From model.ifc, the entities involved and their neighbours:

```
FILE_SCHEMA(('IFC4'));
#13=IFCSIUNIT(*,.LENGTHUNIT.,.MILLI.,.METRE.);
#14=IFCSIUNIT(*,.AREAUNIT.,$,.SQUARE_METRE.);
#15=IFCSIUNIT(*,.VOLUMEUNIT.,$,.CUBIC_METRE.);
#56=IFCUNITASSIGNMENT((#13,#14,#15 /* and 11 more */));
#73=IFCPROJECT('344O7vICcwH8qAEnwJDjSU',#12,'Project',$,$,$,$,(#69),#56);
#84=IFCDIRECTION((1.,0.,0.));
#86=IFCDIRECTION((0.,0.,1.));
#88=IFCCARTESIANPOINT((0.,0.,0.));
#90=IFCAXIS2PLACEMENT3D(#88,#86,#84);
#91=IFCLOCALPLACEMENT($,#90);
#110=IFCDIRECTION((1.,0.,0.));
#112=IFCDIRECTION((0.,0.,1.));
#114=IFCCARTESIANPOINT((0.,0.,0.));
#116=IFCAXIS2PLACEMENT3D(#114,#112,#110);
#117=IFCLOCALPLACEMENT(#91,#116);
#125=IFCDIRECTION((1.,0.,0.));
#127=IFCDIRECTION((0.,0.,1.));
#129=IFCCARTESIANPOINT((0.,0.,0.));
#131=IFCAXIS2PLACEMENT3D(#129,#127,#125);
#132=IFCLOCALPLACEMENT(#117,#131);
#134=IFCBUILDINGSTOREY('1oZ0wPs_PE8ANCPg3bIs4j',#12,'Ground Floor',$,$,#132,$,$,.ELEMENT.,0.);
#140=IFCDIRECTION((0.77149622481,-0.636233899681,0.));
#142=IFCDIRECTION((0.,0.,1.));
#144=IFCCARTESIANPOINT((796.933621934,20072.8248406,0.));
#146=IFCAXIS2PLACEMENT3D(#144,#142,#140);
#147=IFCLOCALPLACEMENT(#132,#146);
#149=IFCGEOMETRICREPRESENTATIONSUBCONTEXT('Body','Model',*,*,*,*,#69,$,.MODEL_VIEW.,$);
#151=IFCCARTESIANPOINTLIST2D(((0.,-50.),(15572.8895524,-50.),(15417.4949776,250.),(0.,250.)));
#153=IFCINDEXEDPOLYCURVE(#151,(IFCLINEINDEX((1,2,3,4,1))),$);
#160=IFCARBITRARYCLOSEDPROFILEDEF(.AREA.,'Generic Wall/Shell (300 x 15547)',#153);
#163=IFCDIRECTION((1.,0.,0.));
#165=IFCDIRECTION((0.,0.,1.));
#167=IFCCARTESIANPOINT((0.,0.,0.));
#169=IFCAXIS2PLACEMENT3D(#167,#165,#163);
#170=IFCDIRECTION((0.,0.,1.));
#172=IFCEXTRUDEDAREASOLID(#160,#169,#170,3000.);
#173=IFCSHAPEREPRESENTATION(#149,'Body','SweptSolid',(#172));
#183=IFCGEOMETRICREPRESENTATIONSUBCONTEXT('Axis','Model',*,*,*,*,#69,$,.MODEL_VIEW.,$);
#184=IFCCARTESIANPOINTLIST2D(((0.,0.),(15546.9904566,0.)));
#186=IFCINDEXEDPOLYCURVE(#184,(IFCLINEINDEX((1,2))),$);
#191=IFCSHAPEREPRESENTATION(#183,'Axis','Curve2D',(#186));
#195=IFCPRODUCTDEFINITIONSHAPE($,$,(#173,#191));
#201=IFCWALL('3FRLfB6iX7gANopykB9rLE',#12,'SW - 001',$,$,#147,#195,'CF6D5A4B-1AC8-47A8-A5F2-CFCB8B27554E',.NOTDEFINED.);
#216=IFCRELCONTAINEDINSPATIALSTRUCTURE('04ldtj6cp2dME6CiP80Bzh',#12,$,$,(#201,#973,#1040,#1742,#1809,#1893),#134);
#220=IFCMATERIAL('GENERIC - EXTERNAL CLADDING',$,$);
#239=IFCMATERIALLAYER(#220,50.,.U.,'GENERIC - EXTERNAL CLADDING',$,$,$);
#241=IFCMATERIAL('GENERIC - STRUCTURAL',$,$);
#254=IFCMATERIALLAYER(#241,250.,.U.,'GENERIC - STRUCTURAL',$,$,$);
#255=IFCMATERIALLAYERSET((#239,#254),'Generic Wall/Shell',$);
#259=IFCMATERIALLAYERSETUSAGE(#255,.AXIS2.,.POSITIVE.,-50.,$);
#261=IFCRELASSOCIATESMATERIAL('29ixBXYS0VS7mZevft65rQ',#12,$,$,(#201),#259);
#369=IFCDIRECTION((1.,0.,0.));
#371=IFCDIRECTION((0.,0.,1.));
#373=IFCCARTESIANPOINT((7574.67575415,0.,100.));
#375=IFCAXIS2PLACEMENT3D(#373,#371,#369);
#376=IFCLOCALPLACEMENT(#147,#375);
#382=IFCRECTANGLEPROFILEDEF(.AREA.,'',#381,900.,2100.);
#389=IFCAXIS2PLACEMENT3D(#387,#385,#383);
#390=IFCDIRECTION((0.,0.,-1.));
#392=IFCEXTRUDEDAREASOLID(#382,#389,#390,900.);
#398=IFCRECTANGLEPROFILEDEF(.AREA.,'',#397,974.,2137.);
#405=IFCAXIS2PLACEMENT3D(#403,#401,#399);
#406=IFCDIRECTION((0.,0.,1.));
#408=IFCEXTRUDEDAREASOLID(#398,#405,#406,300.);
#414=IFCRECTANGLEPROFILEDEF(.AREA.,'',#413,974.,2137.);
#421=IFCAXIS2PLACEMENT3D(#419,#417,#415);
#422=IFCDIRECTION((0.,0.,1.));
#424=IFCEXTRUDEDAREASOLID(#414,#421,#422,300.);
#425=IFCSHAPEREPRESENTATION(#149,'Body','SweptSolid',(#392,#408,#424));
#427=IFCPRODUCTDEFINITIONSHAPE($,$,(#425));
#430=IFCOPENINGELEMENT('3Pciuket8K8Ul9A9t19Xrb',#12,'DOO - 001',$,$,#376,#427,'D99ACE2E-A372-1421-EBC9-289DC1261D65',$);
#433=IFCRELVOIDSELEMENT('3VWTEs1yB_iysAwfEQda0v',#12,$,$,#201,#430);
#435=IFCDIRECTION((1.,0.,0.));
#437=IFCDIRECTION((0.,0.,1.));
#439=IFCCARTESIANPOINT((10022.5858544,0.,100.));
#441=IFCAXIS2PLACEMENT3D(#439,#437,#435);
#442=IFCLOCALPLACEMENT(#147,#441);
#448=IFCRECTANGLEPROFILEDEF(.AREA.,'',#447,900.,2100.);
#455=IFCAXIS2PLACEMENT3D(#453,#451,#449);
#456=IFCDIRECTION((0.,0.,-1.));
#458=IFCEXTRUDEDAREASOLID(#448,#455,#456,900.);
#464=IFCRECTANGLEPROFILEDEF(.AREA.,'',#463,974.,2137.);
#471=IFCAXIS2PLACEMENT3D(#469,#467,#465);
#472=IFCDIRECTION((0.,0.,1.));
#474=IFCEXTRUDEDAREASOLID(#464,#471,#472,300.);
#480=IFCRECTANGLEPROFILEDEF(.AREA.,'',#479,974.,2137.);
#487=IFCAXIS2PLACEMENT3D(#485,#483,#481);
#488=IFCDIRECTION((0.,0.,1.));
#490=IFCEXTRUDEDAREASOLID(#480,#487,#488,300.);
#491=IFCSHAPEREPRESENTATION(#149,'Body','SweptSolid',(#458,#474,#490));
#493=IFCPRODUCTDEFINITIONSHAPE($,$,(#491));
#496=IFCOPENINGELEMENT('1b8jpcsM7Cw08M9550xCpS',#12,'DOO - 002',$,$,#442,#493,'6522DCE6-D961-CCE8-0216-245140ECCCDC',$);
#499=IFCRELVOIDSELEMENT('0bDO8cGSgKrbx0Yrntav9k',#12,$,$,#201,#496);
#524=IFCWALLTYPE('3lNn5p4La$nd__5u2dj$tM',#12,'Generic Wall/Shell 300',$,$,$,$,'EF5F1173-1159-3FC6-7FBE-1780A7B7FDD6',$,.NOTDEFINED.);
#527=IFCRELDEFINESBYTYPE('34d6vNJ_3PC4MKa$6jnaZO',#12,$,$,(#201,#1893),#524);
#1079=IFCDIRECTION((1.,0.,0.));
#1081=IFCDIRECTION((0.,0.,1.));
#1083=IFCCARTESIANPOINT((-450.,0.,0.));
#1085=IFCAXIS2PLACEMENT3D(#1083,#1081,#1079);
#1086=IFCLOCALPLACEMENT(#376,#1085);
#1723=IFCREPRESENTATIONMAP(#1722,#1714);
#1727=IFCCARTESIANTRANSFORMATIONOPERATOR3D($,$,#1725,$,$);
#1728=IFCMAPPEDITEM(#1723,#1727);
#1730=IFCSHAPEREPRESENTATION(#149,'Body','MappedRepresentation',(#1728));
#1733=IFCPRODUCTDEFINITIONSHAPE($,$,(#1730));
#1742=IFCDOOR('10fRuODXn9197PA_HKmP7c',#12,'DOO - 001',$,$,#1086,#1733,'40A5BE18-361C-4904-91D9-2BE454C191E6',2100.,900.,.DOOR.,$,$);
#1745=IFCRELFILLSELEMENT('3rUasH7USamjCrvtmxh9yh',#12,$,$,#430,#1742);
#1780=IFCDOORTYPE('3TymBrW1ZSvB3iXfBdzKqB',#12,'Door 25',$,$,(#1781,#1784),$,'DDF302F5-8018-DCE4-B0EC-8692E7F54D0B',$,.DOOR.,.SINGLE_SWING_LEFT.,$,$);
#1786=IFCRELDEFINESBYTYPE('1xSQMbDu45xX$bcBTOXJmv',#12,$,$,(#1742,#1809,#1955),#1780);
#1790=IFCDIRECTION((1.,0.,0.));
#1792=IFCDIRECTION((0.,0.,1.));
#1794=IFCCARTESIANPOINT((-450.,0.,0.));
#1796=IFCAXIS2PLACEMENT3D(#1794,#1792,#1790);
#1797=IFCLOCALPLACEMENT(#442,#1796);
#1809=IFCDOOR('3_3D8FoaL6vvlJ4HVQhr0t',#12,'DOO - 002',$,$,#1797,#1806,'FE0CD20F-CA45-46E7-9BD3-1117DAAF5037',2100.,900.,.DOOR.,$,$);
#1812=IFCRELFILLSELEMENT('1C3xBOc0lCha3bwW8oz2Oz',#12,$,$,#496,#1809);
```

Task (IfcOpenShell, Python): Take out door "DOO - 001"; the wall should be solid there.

```python
import ifcopenshell
import ifcopenshell.api.feature
import ifcopenshell.api.root
import ifcopenshell.geom
import ifcopenshell.util.shape

model = ifcopenshell.open("model.ifc")
settings = ifcopenshell.geom.settings()


def volume(element):
    """Net volume in cubic metres, openings subtracted."""
    shape = ifcopenshell.geom.create_shape(settings, element)
    return ifcopenshell.util.shape.get_volume(shape.geometry)


door = model.by_guid("10fRuODXn9197PA_HKmP7c")
opening = door.FillsVoids[0].RelatingOpeningElement
wall = opening.VoidsElements[0].RelatingBuildingElement
before = volume(wall)

ifcopenshell.api.root.remove_product(model, product=door)
ifcopenshell.api.feature.remove_feature(model, feature=opening)

after = volume(wall)

print(f"wall volume {before:.3f} -> {after:.3f} m3")

model.write("model_edited.ifc")
```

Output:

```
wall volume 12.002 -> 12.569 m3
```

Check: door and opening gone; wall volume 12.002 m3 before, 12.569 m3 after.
